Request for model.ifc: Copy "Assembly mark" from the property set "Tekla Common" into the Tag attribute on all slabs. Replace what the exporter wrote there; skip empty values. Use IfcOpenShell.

First a look at what the model holds.

```python
import ifcopenshell
import ifcopenshell.util.element

model = ifcopenshell.open("model.ifc")
print(model.schema)
slabs = model.by_type("IfcSlab")
print(len(slabs), "slabs")
for e in slabs[:8]:
    source = ifcopenshell.util.element.get_pset(e, "Tekla Common", "Assembly mark")
    target = e.Tag
    print(e.id(), repr(source), repr(target), sep=" | ")
```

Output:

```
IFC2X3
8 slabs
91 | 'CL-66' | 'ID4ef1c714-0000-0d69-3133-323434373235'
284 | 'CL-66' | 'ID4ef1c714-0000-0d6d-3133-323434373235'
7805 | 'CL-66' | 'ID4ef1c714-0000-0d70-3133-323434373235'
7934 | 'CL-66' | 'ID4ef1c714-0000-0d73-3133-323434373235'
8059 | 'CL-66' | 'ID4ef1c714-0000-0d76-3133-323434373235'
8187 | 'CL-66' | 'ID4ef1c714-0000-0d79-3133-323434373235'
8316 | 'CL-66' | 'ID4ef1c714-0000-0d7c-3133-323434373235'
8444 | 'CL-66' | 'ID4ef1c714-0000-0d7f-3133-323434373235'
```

```python
import ifcopenshell
import ifcopenshell.util.element

model = ifcopenshell.open("model.ifc")

count = 0
for e in model.by_type("IfcSlab"):
    value = ifcopenshell.util.element.get_pset(e, "Tekla Common", "Assembly mark")
    current = e.Tag
    if not value or not value.strip() or current == value:
        continue
    e.Tag = value
    count += 1

print(count, "slabs updated")

model.write("model_updated.ifc")
```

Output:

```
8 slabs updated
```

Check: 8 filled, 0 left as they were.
